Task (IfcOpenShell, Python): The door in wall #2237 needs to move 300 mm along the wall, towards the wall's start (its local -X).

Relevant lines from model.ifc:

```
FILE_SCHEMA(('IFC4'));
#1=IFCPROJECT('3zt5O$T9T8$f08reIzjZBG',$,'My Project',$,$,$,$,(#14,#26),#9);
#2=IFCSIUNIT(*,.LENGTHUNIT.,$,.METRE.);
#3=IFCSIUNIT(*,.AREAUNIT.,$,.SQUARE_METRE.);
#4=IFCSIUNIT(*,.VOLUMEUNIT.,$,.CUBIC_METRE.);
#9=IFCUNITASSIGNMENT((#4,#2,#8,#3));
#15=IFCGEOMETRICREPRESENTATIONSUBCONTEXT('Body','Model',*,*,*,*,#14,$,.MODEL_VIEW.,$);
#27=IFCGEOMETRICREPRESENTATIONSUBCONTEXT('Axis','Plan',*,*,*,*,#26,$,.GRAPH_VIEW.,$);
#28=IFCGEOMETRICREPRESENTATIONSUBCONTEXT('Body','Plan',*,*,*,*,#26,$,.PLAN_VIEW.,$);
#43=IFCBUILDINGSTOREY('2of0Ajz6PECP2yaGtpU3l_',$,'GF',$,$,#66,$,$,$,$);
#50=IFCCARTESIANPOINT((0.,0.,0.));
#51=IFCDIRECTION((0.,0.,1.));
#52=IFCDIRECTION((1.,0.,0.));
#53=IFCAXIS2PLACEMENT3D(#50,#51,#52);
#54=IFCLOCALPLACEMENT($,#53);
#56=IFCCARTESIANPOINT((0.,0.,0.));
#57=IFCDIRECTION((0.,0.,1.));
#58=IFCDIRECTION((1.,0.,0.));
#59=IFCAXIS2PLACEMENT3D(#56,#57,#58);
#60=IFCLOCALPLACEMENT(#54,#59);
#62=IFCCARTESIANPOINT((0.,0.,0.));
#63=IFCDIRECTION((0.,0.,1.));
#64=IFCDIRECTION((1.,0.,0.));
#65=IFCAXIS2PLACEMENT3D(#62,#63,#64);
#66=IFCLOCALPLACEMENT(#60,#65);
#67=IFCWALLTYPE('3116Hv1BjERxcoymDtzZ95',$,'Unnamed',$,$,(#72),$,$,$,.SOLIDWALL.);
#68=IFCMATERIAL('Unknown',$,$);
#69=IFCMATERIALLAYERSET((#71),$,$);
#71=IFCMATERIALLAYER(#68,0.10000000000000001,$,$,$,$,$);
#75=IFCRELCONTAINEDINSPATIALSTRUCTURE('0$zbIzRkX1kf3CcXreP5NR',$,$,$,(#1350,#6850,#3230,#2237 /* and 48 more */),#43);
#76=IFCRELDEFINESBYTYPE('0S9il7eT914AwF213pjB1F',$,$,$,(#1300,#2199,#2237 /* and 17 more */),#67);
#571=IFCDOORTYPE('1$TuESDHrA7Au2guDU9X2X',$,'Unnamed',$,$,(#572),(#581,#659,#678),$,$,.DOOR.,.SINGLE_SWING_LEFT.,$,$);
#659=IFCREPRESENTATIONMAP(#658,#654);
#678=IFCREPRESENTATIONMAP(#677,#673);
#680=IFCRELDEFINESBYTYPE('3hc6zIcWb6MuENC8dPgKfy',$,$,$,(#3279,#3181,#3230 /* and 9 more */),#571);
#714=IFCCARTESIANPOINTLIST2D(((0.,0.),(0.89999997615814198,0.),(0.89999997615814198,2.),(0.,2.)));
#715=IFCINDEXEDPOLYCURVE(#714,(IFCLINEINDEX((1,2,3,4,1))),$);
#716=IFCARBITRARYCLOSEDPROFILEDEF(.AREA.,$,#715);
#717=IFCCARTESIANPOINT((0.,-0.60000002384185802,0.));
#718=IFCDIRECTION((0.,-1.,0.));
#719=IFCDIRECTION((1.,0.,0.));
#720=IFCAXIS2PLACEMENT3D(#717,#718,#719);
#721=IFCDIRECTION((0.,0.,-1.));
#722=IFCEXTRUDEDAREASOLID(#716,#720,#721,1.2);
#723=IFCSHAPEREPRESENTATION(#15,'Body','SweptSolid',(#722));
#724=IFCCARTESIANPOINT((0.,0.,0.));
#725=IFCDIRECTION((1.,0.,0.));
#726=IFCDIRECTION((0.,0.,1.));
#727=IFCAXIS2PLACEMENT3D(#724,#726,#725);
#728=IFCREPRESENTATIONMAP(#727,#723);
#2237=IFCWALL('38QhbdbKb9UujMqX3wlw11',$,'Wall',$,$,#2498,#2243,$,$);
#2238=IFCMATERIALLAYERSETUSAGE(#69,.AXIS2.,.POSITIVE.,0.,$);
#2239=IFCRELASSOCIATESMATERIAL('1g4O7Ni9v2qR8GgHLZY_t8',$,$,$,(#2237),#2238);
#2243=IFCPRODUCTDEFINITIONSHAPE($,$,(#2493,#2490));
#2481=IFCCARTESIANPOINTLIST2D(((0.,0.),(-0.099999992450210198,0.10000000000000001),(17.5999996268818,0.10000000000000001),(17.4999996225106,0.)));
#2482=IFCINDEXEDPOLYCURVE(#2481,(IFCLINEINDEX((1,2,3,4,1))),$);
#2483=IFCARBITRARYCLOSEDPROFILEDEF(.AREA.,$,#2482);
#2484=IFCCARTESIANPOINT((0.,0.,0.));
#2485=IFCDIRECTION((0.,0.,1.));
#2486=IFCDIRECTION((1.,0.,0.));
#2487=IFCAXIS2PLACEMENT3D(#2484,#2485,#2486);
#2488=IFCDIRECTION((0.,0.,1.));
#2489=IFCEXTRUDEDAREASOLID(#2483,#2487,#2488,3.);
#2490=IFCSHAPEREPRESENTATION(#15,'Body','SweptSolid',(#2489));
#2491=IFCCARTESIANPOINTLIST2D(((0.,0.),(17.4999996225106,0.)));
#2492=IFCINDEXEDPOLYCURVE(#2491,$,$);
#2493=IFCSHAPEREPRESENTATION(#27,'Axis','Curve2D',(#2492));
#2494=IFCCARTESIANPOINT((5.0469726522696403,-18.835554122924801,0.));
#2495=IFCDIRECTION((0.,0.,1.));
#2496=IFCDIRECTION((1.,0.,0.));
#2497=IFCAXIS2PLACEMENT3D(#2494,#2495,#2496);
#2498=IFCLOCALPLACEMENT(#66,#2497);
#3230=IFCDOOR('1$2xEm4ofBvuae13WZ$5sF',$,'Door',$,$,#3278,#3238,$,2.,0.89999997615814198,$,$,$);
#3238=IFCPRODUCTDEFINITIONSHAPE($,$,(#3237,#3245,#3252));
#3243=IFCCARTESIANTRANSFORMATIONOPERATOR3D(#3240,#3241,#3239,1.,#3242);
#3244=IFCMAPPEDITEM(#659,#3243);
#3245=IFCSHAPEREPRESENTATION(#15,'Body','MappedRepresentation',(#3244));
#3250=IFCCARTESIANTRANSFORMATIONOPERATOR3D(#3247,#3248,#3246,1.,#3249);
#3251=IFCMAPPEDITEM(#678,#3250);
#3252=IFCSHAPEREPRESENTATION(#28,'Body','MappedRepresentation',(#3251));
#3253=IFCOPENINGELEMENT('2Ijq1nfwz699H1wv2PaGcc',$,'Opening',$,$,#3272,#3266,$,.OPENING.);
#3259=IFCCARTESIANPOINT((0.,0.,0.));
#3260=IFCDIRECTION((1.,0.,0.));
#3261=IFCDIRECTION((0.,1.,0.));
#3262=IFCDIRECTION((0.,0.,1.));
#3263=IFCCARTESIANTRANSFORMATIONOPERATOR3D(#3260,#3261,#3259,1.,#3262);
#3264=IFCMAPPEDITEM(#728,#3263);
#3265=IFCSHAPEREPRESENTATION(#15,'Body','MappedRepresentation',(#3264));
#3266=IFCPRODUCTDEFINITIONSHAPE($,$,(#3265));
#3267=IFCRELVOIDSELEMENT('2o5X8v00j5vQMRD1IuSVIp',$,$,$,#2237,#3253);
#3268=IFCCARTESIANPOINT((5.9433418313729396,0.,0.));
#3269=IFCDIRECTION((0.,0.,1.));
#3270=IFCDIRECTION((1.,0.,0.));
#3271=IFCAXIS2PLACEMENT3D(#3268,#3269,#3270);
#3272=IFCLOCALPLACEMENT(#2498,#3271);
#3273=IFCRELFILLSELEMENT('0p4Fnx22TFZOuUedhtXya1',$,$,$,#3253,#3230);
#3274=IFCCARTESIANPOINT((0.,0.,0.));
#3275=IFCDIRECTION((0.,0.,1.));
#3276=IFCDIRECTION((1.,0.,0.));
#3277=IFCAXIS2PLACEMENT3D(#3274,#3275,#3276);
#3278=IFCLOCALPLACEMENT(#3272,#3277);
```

```python
import ifcopenshell
import ifcopenshell.api.geometry
import ifcopenshell.util.placement

model = ifcopenshell.open("model.ifc")

door = model.by_guid("1$2xEm4ofBvuae13WZ$5sF")
opening = door.FillsVoids[0].RelatingOpeningElement
wall = opening.VoidsElements[0].RelatingBuildingElement

wall_matrix = ifcopenshell.util.placement.get_local_placement(wall.ObjectPlacement)
shift = wall_matrix[:3, 0] * -0.3
before = ifcopenshell.util.placement.get_local_placement(door.ObjectPlacement)[:3, 3].copy()

# The door is placed relative to its opening, so it follows when the opening moves.
matrix = ifcopenshell.util.placement.get_local_placement(opening.ObjectPlacement)
matrix[:3, 3] += shift
ifcopenshell.api.geometry.edit_object_placement(
    model, product=opening, matrix=matrix, is_si=False, should_transform_children=True
)

after = ifcopenshell.util.placement.get_local_placement(door.ObjectPlacement)[:3, 3]
print("door moved by", (after - before).round(3) + 0.0)

model.write("model_v2.ifc")
```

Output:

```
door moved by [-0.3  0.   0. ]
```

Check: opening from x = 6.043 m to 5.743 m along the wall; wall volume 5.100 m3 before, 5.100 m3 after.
